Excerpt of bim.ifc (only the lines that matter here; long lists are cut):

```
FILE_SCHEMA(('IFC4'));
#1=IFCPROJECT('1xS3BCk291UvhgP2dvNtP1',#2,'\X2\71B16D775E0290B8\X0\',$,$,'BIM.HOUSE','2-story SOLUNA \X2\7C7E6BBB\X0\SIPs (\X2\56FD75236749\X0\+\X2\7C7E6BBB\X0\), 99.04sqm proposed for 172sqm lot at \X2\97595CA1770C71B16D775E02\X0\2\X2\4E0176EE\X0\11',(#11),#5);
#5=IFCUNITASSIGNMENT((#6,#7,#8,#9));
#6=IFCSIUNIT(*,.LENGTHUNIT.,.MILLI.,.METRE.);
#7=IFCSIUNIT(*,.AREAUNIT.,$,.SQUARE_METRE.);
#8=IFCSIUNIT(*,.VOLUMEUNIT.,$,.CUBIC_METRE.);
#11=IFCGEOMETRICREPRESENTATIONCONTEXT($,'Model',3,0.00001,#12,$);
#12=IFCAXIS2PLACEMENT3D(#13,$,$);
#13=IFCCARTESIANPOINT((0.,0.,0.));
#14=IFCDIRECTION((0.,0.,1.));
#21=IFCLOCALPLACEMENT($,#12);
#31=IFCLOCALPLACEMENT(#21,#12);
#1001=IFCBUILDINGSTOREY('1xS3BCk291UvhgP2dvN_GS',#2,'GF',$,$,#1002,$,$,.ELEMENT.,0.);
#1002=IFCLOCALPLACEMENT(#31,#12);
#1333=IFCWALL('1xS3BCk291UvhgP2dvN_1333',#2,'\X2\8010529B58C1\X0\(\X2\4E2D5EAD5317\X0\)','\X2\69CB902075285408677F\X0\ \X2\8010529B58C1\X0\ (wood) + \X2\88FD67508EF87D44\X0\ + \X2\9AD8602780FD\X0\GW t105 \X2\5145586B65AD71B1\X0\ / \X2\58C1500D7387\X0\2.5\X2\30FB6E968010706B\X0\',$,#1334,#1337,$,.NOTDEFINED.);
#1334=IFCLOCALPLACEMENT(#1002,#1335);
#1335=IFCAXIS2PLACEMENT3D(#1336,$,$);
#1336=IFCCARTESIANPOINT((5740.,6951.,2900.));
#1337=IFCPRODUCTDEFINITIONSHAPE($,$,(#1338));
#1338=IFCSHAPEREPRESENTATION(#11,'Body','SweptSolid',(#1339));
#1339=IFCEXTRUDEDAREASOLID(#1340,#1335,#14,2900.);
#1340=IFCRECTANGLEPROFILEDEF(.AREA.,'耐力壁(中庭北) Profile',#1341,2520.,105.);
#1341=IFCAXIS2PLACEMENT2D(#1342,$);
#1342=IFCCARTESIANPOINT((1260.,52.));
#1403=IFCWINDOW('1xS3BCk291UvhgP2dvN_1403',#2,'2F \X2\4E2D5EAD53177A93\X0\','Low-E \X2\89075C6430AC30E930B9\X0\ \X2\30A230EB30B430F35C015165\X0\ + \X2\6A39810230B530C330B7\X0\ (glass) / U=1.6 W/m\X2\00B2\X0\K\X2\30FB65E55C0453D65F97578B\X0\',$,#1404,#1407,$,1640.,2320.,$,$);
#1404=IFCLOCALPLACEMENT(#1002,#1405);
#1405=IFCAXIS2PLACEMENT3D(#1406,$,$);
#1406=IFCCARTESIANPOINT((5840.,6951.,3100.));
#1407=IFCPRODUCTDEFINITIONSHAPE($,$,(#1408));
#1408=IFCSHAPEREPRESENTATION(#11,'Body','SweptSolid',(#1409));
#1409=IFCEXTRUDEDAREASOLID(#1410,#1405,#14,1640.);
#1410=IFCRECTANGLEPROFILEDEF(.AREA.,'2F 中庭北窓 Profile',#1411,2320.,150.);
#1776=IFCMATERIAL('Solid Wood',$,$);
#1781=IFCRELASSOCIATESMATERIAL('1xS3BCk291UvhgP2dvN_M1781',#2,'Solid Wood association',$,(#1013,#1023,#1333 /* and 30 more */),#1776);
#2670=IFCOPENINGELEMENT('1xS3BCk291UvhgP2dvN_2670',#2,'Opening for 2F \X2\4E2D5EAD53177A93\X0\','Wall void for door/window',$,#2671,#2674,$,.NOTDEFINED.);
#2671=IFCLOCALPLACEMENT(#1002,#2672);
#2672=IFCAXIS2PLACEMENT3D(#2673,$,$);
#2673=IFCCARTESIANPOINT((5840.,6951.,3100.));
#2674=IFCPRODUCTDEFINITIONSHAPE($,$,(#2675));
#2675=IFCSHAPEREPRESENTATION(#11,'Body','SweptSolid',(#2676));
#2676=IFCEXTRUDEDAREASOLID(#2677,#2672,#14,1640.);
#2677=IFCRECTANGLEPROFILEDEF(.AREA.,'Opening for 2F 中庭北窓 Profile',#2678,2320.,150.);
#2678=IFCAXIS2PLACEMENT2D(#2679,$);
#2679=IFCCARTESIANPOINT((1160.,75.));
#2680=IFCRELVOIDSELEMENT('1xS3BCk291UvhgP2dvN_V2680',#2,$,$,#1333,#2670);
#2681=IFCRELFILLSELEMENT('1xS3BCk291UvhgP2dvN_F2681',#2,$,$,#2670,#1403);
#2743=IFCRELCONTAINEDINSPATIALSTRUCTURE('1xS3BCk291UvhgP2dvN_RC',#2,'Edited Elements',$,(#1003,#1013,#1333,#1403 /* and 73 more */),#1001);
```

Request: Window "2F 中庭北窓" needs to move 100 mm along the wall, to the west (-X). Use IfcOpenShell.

```python
import ifcopenshell
import ifcopenshell.api.geometry
import ifcopenshell.util.placement

model = ifcopenshell.open("bim.ifc")

window = model.by_guid("1xS3BCk291UvhgP2dvN_1403")
opening = window.FillsVoids[0].RelatingOpeningElement
wall = opening.VoidsElements[0].RelatingBuildingElement

wall_matrix = ifcopenshell.util.placement.get_local_placement(wall.ObjectPlacement)
shift = wall_matrix[:3, 0] * -100.0
before = ifcopenshell.util.placement.get_local_placement(window.ObjectPlacement)[:3, 3].copy()

# The window is not placed relative to its opening, so move both.
for product in (opening, window):
    matrix = ifcopenshell.util.placement.get_local_placement(product.ObjectPlacement)
    matrix[:3, 3] += shift
    ifcopenshell.api.geometry.edit_object_placement(model, product=product, matrix=matrix, is_si=False)

after = ifcopenshell.util.placement.get_local_placement(window.ObjectPlacement)[:3, 3]
print("window moved by", (after - before).round(3) + 0.0)

model.write("bim_updated.ifc")
```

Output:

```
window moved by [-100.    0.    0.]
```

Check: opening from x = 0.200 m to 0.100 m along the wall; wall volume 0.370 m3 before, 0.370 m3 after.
